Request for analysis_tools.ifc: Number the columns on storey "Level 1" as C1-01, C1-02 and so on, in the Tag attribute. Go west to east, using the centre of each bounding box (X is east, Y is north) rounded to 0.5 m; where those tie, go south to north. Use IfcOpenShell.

First a look at what the model holds.

```python
import ifcopenshell
import ifcopenshell.util.element
import ifcopenshell.util.placement

model = ifcopenshell.open("analysis_tools.ifc")
print(model.schema)
storey = next(s for s in model.by_type("IfcBuildingStorey") if s.Name == "Level 1")
columns = [e for e in ifcopenshell.util.element.get_decomposition(storey) if e.is_a("IfcColumn")]
for e in sorted(columns, key=lambda e: e.id()):
    origin = ifcopenshell.util.placement.get_local_placement(e.ObjectPlacement)[:3, 3]
    print(e.id(), e.Tag, e.Name, origin.round(2) + 0.0, sep=" | ")
```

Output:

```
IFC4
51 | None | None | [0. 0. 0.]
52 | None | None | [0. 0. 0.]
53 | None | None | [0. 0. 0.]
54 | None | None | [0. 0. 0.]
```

```python
import ifcopenshell
import ifcopenshell.geom
import ifcopenshell.util.element
import ifcopenshell.util.shape

model = ifcopenshell.open("analysis_tools.ifc")
settings = ifcopenshell.geom.settings()
settings.set("use-world-coords", True)


def centre(element):
    shape = ifcopenshell.geom.create_shape(settings, element)
    return ifcopenshell.util.shape.get_bbox_centroid(shape.geometry)


storey = next(s for s in model.by_type("IfcBuildingStorey") if s.Name == "Level 1")
columns = [e for e in ifcopenshell.util.element.get_decomposition(storey) if e.is_a("IfcColumn")]

# Insertion points can sit at a corner or the storey origin, so sort by the geometry (in metres).
centres = {e: centre(e) for e in columns}
columns.sort(key=lambda e: (round(centres[e][0] / 0.5), centres[e][1]))

for i, e in enumerate(columns, start=1):
    number = f"C1-{i:02d}"
    e.Tag = number
    print(e.id(), number)

model.write("analysis_tools_edited.ifc")
```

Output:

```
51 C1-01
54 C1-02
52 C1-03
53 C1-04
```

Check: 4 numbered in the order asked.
